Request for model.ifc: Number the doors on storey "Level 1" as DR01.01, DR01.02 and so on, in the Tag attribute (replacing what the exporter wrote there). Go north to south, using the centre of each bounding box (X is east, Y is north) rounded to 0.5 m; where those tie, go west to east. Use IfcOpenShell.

First a look at what the model holds.

```python
import ifcopenshell
import ifcopenshell.util.element
import ifcopenshell.util.placement

model = ifcopenshell.open("model.ifc")
print(model.schema)
storey = next(s for s in model.by_type("IfcBuildingStorey") if s.Name == "Level 1")
doors = [e for e in ifcopenshell.util.element.get_decomposition(storey) if e.is_a("IfcDoor")]
for e in sorted(doors, key=lambda e: e.id()):
    origin = ifcopenshell.util.placement.get_local_placement(e.ObjectPlacement)[:3, 3]
    print(e.id(), e.Tag, e.Name, origin.round(2) + 0.0, sep=" | ")
```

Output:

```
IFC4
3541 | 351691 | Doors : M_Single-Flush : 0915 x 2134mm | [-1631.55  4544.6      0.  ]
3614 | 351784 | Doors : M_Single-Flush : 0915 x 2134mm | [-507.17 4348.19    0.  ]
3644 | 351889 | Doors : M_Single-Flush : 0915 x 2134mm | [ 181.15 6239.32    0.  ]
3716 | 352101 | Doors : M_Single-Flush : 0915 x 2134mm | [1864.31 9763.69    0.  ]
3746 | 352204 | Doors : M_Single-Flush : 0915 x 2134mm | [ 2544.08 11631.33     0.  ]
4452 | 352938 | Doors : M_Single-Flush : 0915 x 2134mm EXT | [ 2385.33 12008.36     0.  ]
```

```python
import ifcopenshell
import ifcopenshell.geom
import ifcopenshell.util.element
import ifcopenshell.util.shape

model = ifcopenshell.open("model.ifc")
settings = ifcopenshell.geom.settings()
settings.set("use-world-coords", True)


def centre(element):
    shape = ifcopenshell.geom.create_shape(settings, element)
    return ifcopenshell.util.shape.get_bbox_centroid(shape.geometry)


storey = next(s for s in model.by_type("IfcBuildingStorey") if s.Name == "Level 1")
doors = [e for e in ifcopenshell.util.element.get_decomposition(storey) if e.is_a("IfcDoor")]

# Insertion points can sit at a corner or the storey origin, so sort by the geometry (in metres).
centres = {e: centre(e) for e in doors}
doors.sort(key=lambda e: (-round(centres[e][1] / 0.5), centres[e][0]))

for i, e in enumerate(doors, start=1):
    number = f"DR01.{i:02d}"
    e.Tag = number
    print(e.id(), number)

model.write("model_updated.ifc")
```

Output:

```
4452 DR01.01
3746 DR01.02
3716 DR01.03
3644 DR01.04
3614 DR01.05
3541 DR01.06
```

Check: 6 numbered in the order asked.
